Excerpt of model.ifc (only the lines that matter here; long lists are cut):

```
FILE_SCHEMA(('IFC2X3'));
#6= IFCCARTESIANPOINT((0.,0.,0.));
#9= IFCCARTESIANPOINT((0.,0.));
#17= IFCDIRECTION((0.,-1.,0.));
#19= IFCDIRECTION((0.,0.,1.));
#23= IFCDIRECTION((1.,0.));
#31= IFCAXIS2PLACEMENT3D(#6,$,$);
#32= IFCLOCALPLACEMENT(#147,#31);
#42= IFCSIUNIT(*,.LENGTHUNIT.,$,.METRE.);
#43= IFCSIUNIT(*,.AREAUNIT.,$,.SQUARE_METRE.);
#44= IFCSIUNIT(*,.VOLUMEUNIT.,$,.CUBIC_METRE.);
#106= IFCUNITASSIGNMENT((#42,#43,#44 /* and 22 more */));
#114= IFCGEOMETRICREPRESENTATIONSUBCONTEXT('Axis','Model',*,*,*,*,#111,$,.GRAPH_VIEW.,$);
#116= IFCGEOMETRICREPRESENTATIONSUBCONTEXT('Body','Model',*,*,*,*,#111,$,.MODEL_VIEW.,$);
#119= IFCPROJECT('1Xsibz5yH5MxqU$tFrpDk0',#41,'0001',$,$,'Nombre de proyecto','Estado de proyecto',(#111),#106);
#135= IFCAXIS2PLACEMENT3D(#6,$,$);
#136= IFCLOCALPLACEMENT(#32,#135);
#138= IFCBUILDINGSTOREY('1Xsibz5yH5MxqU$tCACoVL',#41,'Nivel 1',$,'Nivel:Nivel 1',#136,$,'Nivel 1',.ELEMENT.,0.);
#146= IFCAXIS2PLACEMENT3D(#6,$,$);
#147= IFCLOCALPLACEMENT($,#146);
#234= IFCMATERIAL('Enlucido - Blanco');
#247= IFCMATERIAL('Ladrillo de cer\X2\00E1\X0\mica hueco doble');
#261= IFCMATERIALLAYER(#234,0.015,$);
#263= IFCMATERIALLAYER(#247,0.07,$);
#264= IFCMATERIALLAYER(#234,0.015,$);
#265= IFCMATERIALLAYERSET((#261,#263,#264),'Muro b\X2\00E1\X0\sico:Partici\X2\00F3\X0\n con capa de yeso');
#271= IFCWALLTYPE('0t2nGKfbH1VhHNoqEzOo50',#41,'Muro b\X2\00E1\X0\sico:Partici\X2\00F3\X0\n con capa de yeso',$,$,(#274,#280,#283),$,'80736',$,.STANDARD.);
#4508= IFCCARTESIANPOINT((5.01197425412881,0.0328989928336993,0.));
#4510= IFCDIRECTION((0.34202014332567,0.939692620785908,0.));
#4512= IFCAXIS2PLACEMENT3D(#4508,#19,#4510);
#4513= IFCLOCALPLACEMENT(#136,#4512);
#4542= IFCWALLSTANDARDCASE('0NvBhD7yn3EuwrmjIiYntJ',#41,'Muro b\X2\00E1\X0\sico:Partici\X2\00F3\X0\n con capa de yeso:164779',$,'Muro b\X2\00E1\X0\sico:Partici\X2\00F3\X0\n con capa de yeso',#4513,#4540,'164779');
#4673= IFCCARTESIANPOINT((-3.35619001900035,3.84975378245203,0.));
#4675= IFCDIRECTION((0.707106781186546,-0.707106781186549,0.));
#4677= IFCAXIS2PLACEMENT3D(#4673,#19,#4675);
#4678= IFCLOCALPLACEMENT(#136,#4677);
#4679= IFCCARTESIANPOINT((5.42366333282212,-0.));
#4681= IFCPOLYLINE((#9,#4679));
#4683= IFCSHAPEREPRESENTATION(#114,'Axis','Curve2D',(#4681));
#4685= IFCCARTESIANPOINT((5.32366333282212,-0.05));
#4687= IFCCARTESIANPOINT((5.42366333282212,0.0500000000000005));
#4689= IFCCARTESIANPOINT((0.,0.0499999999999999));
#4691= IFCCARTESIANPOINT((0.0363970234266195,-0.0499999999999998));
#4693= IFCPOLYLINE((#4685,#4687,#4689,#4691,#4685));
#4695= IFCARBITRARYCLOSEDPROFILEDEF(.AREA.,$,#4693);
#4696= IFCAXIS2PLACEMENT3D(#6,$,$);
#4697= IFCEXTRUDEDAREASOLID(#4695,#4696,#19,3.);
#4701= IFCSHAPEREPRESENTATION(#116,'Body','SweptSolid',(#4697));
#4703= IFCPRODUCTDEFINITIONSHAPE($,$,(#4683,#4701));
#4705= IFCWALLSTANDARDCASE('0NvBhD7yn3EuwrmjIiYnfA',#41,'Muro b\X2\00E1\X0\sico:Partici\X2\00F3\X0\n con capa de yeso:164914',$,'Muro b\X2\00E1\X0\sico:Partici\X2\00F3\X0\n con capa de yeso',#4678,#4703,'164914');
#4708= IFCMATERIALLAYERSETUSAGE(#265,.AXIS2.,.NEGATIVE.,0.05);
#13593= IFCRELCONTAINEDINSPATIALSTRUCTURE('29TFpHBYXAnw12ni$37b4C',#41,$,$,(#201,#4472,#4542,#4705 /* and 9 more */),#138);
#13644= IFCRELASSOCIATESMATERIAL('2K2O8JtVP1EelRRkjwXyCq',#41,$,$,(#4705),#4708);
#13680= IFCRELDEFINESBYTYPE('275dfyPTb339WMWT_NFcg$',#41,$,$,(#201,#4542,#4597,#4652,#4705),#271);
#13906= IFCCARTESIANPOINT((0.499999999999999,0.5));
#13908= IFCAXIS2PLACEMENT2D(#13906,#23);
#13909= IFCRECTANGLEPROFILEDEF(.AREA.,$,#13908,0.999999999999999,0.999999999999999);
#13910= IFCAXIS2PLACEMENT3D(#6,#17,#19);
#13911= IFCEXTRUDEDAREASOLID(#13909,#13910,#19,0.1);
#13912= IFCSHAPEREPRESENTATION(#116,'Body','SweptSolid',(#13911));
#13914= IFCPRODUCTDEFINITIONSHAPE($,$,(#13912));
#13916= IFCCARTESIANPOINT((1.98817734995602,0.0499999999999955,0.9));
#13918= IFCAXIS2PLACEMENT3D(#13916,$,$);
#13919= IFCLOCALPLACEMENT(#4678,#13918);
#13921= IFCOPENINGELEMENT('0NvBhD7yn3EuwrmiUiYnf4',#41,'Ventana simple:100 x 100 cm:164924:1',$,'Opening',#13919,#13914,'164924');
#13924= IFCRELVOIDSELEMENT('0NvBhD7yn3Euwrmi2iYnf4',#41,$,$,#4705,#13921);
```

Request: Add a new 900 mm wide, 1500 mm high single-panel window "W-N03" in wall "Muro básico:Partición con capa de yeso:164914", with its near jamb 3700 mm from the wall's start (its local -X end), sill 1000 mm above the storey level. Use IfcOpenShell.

```python
import numpy as np
import ifcopenshell
import ifcopenshell.api.feature
import ifcopenshell.api.geometry
import ifcopenshell.api.root
import ifcopenshell.api.spatial
import ifcopenshell.api.type
import ifcopenshell.geom
import ifcopenshell.util.element
import ifcopenshell.util.placement
import ifcopenshell.util.representation
import ifcopenshell.util.shape
import ifcopenshell.util.unit

model = ifcopenshell.open("model.ifc")
unit_scale = ifcopenshell.util.unit.calculate_unit_scale(model)
settings = ifcopenshell.geom.settings()


def volume(element):
    """Net volume in cubic metres, openings subtracted."""
    shape = ifcopenshell.geom.create_shape(settings, element)
    return ifcopenshell.util.shape.get_volume(shape.geometry)


wall = model.by_guid("0NvBhD7yn3EuwrmjIiYnfA")
storey = ifcopenshell.util.element.get_container(wall, ifc_class="IfcBuildingStorey")
context = ifcopenshell.util.representation.get_context(model, "Model", "Body", "MODEL_VIEW")
before = volume(wall)

width, height, from_end, sill = 0.9, 1.5, 3.7, 1  # metres

# The wall runs along its own X axis, and the end named is its -X end.
wall_shape = ifcopenshell.geom.create_shape(settings, wall)
x, y, z = ifcopenshell.util.shape.get_vertices(wall_shape.geometry).T
start = x.min() + from_end
face, thickness = float(y.min()), float(y.max() - y.min())
wall_matrix = ifcopenshell.util.placement.get_local_placement(wall.ObjectPlacement)
level = ifcopenshell.util.placement.get_local_placement(storey.ObjectPlacement)[2, 3]


def in_wall(x, y):
    """Placement at x, y metres in the wall's axes, at sill height."""
    matrix = wall_matrix.copy()
    matrix[:, 3] = wall_matrix @ np.array([x / unit_scale, y / unit_scale, 0.0, 1.0])
    matrix[2, 3] = level + sill / unit_scale
    return matrix


# Opening: a box that overshoots both wall faces by 50 mm.
opening = ifcopenshell.api.root.create_entity(model, ifc_class="IfcOpeningElement")
box = ifcopenshell.api.geometry.add_wall_representation(
    model, context=context, length=width, height=height, thickness=thickness + 0.1
)
ifcopenshell.api.geometry.assign_representation(model, product=opening, representation=box)
ifcopenshell.api.geometry.edit_object_placement(model, product=opening, matrix=in_wall(start, face - 0.05), is_si=False)
ifcopenshell.api.feature.add_feature(model, feature=opening, element=wall)

window = ifcopenshell.api.root.create_entity(model, ifc_class="IfcWindow", name="W-N03")
window.OverallWidth, window.OverallHeight = width / unit_scale, height / unit_scale
body = ifcopenshell.api.geometry.add_window_representation(
    model,
    context=context,
    overall_width=window.OverallWidth,
    overall_height=window.OverallHeight,
    partition_type="SINGLE_PANEL",
)
ifcopenshell.api.geometry.assign_representation(model, product=window, representation=body)
ifcopenshell.api.spatial.assign_container(model, products=[window], relating_structure=storey)
fills = ifcopenshell.api.feature.add_filling(model, opening=opening, element=window)
fills.OwnerHistory = window.OwnerHistory  # required in IFC2X3

# IFC2X3 keeps the operation on the window style.
style = ifcopenshell.api.root.create_entity(model, ifc_class="IfcWindowStyle", name="W-N03")
style.OperationType, style.ConstructionType = "SINGLE_PANEL", "NOTDEFINED"
style.ParameterTakesPrecedence = style.Sizeable = False
ifcopenshell.api.type.assign_type(model, related_objects=[window], relating_type=style)

# Centre the window in the wall's thickness.
ifcopenshell.api.geometry.edit_object_placement(model, product=window, matrix=in_wall(start, face), is_si=False)
window_shape = ifcopenshell.geom.create_shape(settings, window)
depth = ifcopenshell.util.shape.get_vertices(window_shape.geometry)[:, 1]
offset = face + thickness / 2 - (depth.min() + depth.max()) / 2
ifcopenshell.api.geometry.edit_object_placement(model, product=window, matrix=in_wall(start, offset), is_si=False)

after = volume(wall)

print(f"wall volume {before:.3f} -> {after:.3f} m3")

model.write("model_updated.ifc")
```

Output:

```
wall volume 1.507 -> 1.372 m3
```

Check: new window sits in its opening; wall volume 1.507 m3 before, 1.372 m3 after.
